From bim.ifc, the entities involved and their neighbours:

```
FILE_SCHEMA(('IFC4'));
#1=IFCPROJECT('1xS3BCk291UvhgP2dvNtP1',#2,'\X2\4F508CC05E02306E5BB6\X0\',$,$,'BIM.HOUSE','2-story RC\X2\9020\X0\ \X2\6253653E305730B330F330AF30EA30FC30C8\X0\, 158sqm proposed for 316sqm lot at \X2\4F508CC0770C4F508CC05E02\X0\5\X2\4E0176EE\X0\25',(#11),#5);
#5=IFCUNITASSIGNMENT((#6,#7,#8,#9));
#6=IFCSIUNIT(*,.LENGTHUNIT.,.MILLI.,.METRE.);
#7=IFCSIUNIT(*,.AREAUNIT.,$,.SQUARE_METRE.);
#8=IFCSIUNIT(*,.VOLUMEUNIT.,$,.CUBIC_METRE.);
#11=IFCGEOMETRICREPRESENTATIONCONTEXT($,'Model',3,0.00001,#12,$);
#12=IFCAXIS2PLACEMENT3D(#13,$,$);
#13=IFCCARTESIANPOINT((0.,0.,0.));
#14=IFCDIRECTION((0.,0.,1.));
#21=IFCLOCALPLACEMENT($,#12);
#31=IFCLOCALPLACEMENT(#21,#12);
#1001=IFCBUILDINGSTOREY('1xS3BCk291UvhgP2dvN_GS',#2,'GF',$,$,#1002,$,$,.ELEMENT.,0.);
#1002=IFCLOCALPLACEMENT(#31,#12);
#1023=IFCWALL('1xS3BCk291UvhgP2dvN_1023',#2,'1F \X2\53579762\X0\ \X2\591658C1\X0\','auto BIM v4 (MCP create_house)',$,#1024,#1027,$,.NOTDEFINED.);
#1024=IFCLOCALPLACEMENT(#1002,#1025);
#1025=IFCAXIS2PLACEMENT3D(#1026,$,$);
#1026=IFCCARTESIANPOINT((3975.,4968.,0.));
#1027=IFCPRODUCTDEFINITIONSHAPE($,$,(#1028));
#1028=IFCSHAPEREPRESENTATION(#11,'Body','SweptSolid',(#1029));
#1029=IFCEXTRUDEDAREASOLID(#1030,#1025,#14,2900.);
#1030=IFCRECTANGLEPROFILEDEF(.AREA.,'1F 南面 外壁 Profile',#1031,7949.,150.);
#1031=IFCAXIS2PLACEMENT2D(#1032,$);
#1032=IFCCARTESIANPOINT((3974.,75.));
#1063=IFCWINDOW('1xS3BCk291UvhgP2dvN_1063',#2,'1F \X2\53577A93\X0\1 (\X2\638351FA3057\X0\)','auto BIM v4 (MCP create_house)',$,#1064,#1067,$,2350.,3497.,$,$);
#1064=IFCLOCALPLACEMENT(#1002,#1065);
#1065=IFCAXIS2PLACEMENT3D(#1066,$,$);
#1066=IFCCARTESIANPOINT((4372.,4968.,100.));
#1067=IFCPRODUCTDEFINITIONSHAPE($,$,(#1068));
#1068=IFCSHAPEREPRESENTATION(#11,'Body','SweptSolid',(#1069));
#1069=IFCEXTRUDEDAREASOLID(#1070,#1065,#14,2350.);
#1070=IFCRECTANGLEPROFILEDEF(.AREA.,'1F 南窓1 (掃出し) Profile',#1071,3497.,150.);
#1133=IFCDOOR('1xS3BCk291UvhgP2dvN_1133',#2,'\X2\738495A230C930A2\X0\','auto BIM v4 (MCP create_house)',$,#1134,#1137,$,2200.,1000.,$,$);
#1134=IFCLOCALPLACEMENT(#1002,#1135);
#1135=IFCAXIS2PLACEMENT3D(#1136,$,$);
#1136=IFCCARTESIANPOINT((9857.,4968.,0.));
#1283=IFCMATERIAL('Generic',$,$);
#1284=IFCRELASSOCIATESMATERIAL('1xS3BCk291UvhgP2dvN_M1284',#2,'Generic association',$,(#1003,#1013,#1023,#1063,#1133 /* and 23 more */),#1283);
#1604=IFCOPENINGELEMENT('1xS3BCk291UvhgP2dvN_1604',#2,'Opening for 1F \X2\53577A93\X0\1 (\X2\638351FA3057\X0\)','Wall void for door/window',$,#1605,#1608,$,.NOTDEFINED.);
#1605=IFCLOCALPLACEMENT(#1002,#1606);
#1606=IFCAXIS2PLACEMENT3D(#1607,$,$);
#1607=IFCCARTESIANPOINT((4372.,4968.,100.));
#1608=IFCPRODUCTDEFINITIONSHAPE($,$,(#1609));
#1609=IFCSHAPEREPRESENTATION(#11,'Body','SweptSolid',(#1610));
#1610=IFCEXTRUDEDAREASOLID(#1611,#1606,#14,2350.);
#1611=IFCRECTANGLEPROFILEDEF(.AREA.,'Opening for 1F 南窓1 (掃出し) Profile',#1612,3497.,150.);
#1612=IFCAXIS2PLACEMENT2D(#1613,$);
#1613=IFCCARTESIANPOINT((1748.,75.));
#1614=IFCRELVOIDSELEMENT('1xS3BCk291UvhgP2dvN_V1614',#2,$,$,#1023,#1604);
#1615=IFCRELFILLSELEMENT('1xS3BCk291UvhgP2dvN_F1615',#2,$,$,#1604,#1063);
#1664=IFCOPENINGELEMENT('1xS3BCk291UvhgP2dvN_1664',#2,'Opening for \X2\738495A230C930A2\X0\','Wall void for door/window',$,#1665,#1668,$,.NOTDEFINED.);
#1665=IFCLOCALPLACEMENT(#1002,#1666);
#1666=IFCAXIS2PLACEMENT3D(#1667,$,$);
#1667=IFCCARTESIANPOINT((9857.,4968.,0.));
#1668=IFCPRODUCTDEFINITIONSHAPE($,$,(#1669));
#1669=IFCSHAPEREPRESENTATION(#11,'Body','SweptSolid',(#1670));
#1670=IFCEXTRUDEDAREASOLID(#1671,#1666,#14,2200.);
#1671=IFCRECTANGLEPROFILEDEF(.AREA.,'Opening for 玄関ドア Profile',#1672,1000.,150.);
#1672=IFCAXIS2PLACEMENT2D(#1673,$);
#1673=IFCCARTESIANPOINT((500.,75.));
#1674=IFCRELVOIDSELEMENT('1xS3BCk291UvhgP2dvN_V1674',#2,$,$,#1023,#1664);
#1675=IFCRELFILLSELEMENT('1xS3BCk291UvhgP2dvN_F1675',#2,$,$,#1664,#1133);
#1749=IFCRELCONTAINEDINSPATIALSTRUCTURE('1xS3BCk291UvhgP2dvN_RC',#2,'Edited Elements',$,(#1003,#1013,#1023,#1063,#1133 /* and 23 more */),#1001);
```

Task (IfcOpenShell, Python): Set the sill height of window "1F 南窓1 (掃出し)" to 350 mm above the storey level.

```python
import numpy as np
import ifcopenshell
import ifcopenshell.api.geometry
import ifcopenshell.geom
import ifcopenshell.util.element
import ifcopenshell.util.placement
import ifcopenshell.util.shape
import ifcopenshell.util.unit

model = ifcopenshell.open("bim.ifc")
unit_scale = ifcopenshell.util.unit.calculate_unit_scale(model)

window = model.by_id(1063)
opening = window.FillsVoids[0].RelatingOpeningElement
storey = ifcopenshell.util.element.get_container(window, ifc_class="IfcBuildingStorey")
level = ifcopenshell.util.placement.get_local_placement(storey.ObjectPlacement)[2, 3]

# The opening's origin need not be at the sill, so measure its lowest point.
shape = ifcopenshell.geom.create_shape(ifcopenshell.geom.settings(), opening)
bottom = ifcopenshell.util.shape.get_shape_bottom_elevation(shape, shape.geometry) / unit_scale
dz = level + 350.0 - bottom

shift = np.array([0.0, 0.0, dz])
# The window is not placed relative to its opening, so move both.
for product in (opening, window):
    matrix = ifcopenshell.util.placement.get_local_placement(product.ObjectPlacement)
    matrix[:3, 3] += shift
    ifcopenshell.api.geometry.edit_object_placement(model, product=product, matrix=matrix, is_si=False)

print(f"moved by {dz * unit_scale:+.3f} m")

model.write("bim_edited.ifc")
```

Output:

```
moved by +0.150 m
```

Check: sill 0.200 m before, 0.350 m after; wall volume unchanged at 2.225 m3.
